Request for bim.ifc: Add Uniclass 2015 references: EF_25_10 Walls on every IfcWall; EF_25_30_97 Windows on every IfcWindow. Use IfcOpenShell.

First a look at what the model holds.

```python
import ifcopenshell

model = ifcopenshell.open("bim.ifc")
print(model.schema)
print("classifications:", [c.Name for c in model.by_type("IfcClassification")])
for ifc_class in ("IfcDoor", "IfcRoof", "IfcStair", "IfcWall", "IfcWindow"):
    print(ifc_class, len(model.by_type(ifc_class)))
```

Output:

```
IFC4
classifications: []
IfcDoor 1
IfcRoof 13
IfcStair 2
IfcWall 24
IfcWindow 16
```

```python
import ifcopenshell
import ifcopenshell.api.classification

model = ifcopenshell.open("bim.ifc")

system = ifcopenshell.api.classification.add_classification(model, classification="Uniclass 2015")

codes = {
    "IfcWall": ("EF_25_10", "Walls"),
    "IfcWindow": ("EF_25_30_97", "Windows"),
}
for ifc_class, (code, name) in codes.items():
    products = model.by_type(ifc_class)
    ifcopenshell.api.classification.add_reference(
        model, products=products, classification=system, identification=code, name=name
    )
    print(code, len(products))

model.write("bim_rev.ifc")
```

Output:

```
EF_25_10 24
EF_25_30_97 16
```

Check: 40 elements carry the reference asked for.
